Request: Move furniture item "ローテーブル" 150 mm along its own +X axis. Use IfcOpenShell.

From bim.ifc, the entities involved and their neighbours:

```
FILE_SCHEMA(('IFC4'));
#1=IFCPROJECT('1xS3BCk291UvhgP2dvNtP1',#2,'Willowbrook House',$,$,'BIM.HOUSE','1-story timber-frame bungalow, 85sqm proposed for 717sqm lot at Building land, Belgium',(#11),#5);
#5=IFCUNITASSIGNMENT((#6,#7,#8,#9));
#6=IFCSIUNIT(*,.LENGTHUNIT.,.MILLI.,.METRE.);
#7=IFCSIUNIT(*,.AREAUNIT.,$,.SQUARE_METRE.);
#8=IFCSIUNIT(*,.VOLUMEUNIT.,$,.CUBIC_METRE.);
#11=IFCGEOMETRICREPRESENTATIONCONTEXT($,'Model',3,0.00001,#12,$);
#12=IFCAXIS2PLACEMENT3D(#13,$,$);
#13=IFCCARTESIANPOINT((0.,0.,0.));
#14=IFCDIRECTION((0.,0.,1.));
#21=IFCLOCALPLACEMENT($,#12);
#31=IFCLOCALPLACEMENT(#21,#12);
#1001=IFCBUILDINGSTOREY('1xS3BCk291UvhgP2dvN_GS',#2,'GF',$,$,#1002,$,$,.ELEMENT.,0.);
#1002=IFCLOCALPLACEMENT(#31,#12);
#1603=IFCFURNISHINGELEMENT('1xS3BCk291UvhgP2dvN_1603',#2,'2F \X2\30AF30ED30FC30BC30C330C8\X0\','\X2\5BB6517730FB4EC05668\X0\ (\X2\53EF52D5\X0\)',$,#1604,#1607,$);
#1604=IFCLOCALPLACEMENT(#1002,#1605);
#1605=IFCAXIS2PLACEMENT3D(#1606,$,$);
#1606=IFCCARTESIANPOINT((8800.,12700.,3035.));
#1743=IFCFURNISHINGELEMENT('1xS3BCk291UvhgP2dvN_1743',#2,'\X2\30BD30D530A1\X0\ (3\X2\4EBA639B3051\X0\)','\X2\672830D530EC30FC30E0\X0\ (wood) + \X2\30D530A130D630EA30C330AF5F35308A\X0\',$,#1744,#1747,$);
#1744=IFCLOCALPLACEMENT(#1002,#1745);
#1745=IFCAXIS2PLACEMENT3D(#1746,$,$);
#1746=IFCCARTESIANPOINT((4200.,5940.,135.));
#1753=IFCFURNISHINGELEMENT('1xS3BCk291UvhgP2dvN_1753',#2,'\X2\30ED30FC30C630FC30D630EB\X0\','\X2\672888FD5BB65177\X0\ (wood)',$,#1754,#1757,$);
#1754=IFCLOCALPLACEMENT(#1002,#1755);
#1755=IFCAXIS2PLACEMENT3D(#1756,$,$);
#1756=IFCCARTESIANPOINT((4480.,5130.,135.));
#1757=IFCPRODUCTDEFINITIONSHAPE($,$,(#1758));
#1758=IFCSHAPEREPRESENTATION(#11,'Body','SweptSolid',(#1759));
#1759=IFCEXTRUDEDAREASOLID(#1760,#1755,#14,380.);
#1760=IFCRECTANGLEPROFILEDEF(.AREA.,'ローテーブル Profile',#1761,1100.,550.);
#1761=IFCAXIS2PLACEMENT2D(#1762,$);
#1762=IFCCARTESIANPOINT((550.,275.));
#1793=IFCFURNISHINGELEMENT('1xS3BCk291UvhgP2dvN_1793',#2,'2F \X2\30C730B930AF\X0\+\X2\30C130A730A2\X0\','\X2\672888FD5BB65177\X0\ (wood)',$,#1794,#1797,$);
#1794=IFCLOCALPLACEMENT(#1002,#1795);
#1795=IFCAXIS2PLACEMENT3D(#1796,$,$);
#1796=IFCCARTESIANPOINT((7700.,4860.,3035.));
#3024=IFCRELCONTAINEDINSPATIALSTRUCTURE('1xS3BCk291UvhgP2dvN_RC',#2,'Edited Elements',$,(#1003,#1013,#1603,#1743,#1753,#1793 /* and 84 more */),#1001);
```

```python
import ifcopenshell
import ifcopenshell.api.geometry
import ifcopenshell.util.placement

model = ifcopenshell.open("bim.ifc")

item = model.by_guid("1xS3BCk291UvhgP2dvN_1753")
matrix = ifcopenshell.util.placement.get_local_placement(item.ObjectPlacement)
matrix[:3, 3] += matrix[:3, 0] * 150.0
ifcopenshell.api.geometry.edit_object_placement(model, product=item, matrix=matrix, is_si=False)

print(ifcopenshell.util.placement.get_local_placement(item.ObjectPlacement).round(3) + 0.0)

model.write("bim-out.ifc")
```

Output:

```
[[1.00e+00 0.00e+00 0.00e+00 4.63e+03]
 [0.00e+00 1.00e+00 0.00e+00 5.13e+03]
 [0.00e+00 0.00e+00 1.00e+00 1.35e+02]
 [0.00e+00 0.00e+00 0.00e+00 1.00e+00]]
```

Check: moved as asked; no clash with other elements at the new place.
